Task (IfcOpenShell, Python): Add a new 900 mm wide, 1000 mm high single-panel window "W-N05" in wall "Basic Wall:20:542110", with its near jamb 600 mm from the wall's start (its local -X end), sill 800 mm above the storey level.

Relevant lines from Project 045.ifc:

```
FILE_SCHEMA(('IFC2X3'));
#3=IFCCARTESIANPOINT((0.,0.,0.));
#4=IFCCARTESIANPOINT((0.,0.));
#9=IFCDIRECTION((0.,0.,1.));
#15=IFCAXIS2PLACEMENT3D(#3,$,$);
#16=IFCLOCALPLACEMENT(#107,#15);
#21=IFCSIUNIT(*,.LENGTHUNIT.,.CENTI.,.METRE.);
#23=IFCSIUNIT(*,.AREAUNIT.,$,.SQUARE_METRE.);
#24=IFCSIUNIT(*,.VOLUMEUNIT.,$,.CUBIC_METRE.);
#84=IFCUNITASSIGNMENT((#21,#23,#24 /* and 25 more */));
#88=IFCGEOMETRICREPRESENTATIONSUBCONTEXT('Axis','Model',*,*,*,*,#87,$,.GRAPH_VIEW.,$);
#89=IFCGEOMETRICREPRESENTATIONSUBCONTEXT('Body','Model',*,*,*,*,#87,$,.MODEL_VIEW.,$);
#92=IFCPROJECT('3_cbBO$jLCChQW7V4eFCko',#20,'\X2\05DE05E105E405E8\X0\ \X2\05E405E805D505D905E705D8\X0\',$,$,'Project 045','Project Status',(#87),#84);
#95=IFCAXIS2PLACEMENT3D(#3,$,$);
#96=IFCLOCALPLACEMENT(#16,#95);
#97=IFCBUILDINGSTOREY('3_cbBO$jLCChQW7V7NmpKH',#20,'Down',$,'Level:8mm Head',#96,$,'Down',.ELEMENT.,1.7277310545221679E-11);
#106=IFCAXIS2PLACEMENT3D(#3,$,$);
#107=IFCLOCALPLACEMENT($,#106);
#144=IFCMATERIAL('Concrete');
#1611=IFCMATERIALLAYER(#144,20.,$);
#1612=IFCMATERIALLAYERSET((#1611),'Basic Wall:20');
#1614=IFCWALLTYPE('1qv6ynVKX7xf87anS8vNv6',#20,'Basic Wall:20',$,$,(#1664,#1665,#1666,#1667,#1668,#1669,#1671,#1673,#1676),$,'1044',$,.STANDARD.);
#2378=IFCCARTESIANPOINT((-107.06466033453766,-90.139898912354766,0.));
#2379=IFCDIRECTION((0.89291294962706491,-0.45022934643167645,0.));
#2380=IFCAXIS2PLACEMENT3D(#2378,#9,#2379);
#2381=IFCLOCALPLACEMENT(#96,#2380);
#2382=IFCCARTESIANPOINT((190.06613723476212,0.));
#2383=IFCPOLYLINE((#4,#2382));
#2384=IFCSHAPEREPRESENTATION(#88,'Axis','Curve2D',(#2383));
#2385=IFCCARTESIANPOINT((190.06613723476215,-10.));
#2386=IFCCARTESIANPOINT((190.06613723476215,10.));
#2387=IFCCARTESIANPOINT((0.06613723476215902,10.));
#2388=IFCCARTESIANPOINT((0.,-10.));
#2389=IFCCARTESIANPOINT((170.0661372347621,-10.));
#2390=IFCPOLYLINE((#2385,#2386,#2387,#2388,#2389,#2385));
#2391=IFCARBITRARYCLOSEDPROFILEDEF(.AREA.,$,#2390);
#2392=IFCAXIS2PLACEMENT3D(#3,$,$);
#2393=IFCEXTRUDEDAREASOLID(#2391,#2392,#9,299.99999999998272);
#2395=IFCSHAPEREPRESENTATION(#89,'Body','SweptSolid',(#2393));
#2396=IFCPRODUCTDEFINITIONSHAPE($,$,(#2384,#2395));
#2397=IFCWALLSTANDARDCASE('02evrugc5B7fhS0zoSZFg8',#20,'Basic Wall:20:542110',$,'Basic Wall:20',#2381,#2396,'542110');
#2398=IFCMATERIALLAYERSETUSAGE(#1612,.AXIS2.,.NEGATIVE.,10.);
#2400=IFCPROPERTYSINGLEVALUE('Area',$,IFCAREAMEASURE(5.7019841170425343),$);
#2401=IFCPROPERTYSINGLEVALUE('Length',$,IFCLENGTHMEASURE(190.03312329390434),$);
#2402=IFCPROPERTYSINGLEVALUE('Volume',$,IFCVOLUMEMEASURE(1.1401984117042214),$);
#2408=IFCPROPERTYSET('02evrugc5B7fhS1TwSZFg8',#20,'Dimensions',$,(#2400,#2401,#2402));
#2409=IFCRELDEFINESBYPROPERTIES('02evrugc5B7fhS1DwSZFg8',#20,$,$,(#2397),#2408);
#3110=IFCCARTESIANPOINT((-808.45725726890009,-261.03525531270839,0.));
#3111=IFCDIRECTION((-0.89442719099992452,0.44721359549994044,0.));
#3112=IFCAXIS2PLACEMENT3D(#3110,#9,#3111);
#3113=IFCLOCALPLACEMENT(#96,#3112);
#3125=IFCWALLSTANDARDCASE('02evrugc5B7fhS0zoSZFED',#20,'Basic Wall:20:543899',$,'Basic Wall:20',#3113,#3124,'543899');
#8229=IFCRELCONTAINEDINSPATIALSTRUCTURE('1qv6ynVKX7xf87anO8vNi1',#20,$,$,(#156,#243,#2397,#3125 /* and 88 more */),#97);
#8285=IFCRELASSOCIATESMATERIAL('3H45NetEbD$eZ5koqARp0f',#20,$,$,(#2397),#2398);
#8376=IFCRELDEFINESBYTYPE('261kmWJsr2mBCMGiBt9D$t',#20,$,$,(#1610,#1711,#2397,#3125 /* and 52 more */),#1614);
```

```python
import numpy as np
import ifcopenshell
import ifcopenshell.api.feature
import ifcopenshell.api.geometry
import ifcopenshell.api.pset
import ifcopenshell.api.root
import ifcopenshell.api.spatial
import ifcopenshell.api.type
import ifcopenshell.geom
import ifcopenshell.util.element
import ifcopenshell.util.placement
import ifcopenshell.util.representation
import ifcopenshell.util.shape
import ifcopenshell.util.unit

model = ifcopenshell.open("Project 045.ifc")
unit_scale = ifcopenshell.util.unit.calculate_unit_scale(model)
area_scale = ifcopenshell.util.unit.calculate_unit_scale(model, "AREAUNIT")
volume_scale = ifcopenshell.util.unit.calculate_unit_scale(model, "VOLUMEUNIT")
settings = ifcopenshell.geom.settings()


def volume(element):
    """Net volume in cubic metres, openings subtracted."""
    shape = ifcopenshell.geom.create_shape(settings, element)
    return ifcopenshell.util.shape.get_volume(shape.geometry)


wall = model.by_id(2397)
storey = ifcopenshell.util.element.get_container(wall, ifc_class="IfcBuildingStorey")
context = ifcopenshell.util.representation.get_context(model, "Model", "Body", "MODEL_VIEW")
before = volume(wall)

width, height, from_end, sill = 0.9, 1, 0.6, 0.8  # metres

# The wall runs along its own X axis, and the end named is its -X end.
wall_shape = ifcopenshell.geom.create_shape(settings, wall)
x, y, z = ifcopenshell.util.shape.get_vertices(wall_shape.geometry).T
start = x.min() + from_end
face, thickness = float(y.min()), float(y.max() - y.min())
wall_matrix = ifcopenshell.util.placement.get_local_placement(wall.ObjectPlacement)
level = ifcopenshell.util.placement.get_local_placement(storey.ObjectPlacement)[2, 3]


def in_wall(x, y):
    """Placement at x, y metres in the wall's axes, at sill height."""
    matrix = wall_matrix.copy()
    matrix[:, 3] = wall_matrix @ np.array([x / unit_scale, y / unit_scale, 0.0, 1.0])
    matrix[2, 3] = level + sill / unit_scale
    return matrix


# Opening: a box that overshoots both wall faces by 50 mm.
opening = ifcopenshell.api.root.create_entity(model, ifc_class="IfcOpeningElement")
box = ifcopenshell.api.geometry.add_wall_representation(
    model, context=context, length=width, height=height, thickness=thickness + 0.1
)
ifcopenshell.api.geometry.assign_representation(model, product=opening, representation=box)
ifcopenshell.api.geometry.edit_object_placement(model, product=opening, matrix=in_wall(start, face - 0.05), is_si=False)
ifcopenshell.api.feature.add_feature(model, feature=opening, element=wall)

window = ifcopenshell.api.root.create_entity(model, ifc_class="IfcWindow", name="W-N05")
window.OverallWidth, window.OverallHeight = width / unit_scale, height / unit_scale
body = ifcopenshell.api.geometry.add_window_representation(
    model,
    context=context,
    overall_width=window.OverallWidth,
    overall_height=window.OverallHeight,
    partition_type="SINGLE_PANEL",
)
ifcopenshell.api.geometry.assign_representation(model, product=window, representation=body)
ifcopenshell.api.spatial.assign_container(model, products=[window], relating_structure=storey)
fills = ifcopenshell.api.feature.add_filling(model, opening=opening, element=window)
fills.OwnerHistory = window.OwnerHistory  # required in IFC2X3

# IFC2X3 keeps the operation on the window style.
style = ifcopenshell.api.root.create_entity(model, ifc_class="IfcWindowStyle", name="W-N05")
style.OperationType, style.ConstructionType = "SINGLE_PANEL", "NOTDEFINED"
style.ParameterTakesPrecedence = style.Sizeable = False
ifcopenshell.api.type.assign_type(model, related_objects=[window], relating_type=style)

# Centre the window in the wall's thickness.
ifcopenshell.api.geometry.edit_object_placement(model, product=window, matrix=in_wall(start, face), is_si=False)
window_shape = ifcopenshell.geom.create_shape(settings, window)
depth = ifcopenshell.util.shape.get_vertices(window_shape.geometry)[:, 1]
offset = face + thickness / 2 - (depth.min() + depth.max()) / 2
ifcopenshell.api.geometry.edit_object_placement(model, product=window, matrix=in_wall(start, offset), is_si=False)

after = volume(wall)

# Update the wall's stored quantities.
pset = model.by_id(ifcopenshell.util.element.get_pset(wall, "Dimensions", should_inherit=False)["id"])
ifcopenshell.api.pset.edit_pset(model, pset=pset, properties={
    "Area": model.create_entity("IfcAreaMeasure", after / thickness / area_scale),
    "Volume": model.create_entity("IfcVolumeMeasure", after / volume_scale),
})

print(f"wall volume {before:.3f} -> {after:.3f} m3")

model.write("Project 045_edited.ifc")
```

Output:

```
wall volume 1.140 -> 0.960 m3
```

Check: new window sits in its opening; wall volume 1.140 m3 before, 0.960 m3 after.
